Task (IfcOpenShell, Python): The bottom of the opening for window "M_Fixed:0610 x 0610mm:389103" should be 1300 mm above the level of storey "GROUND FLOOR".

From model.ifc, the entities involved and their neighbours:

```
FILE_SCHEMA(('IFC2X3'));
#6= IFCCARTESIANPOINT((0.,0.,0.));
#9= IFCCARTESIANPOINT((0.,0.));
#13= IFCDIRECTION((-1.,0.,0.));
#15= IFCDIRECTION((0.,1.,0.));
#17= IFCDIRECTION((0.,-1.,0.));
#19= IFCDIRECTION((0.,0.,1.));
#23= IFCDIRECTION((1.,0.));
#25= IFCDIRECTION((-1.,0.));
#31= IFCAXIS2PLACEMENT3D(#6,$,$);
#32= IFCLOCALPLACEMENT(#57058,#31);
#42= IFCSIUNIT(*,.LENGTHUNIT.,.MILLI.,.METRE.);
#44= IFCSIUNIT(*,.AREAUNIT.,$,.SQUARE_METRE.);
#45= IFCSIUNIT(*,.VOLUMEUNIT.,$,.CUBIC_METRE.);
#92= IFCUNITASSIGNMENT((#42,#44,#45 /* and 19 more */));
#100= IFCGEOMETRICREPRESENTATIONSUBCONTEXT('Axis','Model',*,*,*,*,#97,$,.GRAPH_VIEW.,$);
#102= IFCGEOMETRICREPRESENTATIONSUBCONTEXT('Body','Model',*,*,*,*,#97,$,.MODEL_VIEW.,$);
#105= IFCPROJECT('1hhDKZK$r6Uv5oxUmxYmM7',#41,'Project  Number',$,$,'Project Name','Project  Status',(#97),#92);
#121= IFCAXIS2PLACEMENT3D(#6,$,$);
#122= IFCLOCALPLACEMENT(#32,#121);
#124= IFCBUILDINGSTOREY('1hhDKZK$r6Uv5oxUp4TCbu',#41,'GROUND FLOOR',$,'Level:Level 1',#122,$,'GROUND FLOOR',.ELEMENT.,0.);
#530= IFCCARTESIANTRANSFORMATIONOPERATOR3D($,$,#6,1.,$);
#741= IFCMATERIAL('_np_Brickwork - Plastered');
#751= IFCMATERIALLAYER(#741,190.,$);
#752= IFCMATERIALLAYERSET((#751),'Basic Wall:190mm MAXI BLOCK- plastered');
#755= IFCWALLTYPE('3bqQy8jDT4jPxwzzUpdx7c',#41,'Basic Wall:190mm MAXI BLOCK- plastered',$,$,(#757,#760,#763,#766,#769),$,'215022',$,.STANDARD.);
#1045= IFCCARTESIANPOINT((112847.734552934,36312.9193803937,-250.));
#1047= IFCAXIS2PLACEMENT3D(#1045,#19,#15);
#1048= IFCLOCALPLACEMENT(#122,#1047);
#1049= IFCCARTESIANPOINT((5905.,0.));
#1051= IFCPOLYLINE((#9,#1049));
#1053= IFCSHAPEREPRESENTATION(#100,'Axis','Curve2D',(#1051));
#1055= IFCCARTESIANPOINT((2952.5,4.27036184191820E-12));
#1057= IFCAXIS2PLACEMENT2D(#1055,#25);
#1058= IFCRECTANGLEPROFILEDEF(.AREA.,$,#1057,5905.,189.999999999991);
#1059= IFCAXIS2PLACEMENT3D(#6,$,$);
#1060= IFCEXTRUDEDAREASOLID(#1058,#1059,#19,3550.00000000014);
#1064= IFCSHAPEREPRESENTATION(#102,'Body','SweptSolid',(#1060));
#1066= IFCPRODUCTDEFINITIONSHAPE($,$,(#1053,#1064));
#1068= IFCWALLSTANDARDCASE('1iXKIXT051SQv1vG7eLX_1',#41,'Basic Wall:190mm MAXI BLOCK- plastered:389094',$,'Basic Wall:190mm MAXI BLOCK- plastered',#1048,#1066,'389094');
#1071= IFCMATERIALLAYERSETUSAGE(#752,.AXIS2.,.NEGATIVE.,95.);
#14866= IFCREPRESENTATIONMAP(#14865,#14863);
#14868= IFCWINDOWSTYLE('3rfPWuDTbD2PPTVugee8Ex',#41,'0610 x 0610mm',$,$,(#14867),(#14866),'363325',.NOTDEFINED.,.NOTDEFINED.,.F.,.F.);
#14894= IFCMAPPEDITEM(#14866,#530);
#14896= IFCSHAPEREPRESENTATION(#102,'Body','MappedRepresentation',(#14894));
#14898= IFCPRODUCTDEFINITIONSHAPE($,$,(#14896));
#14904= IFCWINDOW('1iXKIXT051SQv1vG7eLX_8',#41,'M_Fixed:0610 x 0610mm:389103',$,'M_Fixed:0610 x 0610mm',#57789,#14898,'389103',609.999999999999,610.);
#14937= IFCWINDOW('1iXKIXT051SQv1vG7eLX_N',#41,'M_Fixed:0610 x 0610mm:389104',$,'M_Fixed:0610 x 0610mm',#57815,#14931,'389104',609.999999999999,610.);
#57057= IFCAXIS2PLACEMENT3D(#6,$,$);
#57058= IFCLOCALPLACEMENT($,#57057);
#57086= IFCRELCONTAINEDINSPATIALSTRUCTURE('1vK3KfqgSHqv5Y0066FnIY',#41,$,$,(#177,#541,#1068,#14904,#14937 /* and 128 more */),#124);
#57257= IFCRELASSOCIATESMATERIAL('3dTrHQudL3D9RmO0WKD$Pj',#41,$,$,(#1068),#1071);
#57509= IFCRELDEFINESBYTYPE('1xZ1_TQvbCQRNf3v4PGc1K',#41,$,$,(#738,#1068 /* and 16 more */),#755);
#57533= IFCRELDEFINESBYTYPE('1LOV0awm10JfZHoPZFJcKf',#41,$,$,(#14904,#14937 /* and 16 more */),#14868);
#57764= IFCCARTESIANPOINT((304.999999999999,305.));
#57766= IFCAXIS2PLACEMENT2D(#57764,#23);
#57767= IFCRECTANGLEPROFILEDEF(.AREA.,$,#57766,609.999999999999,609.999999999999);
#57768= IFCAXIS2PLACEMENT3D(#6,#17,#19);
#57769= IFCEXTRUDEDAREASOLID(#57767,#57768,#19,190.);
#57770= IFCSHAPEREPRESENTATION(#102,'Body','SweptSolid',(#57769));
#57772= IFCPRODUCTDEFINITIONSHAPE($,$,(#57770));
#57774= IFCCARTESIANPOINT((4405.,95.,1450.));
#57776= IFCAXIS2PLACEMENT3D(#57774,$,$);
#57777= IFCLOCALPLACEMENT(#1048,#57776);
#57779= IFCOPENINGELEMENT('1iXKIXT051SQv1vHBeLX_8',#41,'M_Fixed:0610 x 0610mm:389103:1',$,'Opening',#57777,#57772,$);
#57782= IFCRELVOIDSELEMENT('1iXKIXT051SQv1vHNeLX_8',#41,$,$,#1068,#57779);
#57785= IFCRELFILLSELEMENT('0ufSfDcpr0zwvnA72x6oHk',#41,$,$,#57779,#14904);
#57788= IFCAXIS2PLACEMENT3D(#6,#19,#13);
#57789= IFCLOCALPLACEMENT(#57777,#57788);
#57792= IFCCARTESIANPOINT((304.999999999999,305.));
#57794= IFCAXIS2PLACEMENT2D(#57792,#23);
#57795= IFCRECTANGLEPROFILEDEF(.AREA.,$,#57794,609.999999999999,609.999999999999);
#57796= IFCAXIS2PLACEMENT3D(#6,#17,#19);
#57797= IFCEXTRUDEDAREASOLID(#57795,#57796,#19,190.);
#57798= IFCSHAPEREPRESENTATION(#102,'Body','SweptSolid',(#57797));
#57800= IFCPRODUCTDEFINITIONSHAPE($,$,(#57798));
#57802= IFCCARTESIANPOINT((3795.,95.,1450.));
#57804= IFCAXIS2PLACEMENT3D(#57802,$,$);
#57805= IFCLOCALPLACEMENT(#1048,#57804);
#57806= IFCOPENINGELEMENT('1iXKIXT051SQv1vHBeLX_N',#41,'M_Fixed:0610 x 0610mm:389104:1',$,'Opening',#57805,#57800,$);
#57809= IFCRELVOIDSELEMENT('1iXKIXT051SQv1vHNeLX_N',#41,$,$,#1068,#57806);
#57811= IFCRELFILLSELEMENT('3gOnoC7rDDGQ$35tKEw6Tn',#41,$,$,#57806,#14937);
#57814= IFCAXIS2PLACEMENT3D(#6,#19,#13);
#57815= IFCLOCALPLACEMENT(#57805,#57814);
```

```python
import numpy as np
import ifcopenshell
import ifcopenshell.api.geometry
import ifcopenshell.geom
import ifcopenshell.util.element
import ifcopenshell.util.placement
import ifcopenshell.util.shape
import ifcopenshell.util.unit

model = ifcopenshell.open("model.ifc")
unit_scale = ifcopenshell.util.unit.calculate_unit_scale(model)

window = model.by_guid("1iXKIXT051SQv1vG7eLX_8")
opening = window.FillsVoids[0].RelatingOpeningElement
storey = ifcopenshell.util.element.get_container(window, ifc_class="IfcBuildingStorey")
level = ifcopenshell.util.placement.get_local_placement(storey.ObjectPlacement)[2, 3]

# The opening's origin need not be at the sill, so measure its lowest point.
shape = ifcopenshell.geom.create_shape(ifcopenshell.geom.settings(), opening)
bottom = ifcopenshell.util.shape.get_shape_bottom_elevation(shape, shape.geometry) / unit_scale
dz = level + 1300.0 - bottom

shift = np.array([0.0, 0.0, dz])
# The window is placed relative to its opening, so it follows when the opening moves.
matrix = ifcopenshell.util.placement.get_local_placement(opening.ObjectPlacement)
matrix[:3, 3] += shift
ifcopenshell.api.geometry.edit_object_placement(
    model, product=opening, matrix=matrix, is_si=False, should_transform_children=True
)

print(f"moved by {dz * unit_scale:+.3f} m")

model.write("model-out.ifc")
```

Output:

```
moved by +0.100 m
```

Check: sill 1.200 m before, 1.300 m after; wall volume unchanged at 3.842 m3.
